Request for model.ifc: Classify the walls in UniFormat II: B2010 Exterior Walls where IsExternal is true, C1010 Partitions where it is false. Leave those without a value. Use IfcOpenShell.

First a look at what the model holds.

```python
import ifcopenshell
import ifcopenshell.util.element

model = ifcopenshell.open("model.ifc")
print(model.schema)
print("classifications:", [c.Name for c in model.by_type("IfcClassification")])
values = [ifcopenshell.util.element.get_pset(e, "Pset_WallCommon", "IsExternal") for e in model.by_type("IfcWall")]
for value in (True, False, None):
    print("IsExternal", value, values.count(value))
```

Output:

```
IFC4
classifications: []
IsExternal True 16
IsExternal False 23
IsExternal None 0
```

```python
import ifcopenshell
import ifcopenshell.api.classification
import ifcopenshell.util.element

model = ifcopenshell.open("model.ifc")

system = ifcopenshell.api.classification.add_classification(model, classification="UniFormat II")

walls = model.by_type("IfcWall")
external = {e: ifcopenshell.util.element.get_pset(e, "Pset_WallCommon", "IsExternal") for e in walls}
for flag, code, name in ((True, "B2010", "Exterior Walls"), (False, "C1010", "Partitions")):
    products = [e for e in walls if external[e] is flag]
    ifcopenshell.api.classification.add_reference(
        model, products=products, classification=system, identification=code, name=name
    )
    print(code, len(products))

model.write("model_v2.ifc")
```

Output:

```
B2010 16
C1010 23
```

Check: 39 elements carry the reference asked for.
